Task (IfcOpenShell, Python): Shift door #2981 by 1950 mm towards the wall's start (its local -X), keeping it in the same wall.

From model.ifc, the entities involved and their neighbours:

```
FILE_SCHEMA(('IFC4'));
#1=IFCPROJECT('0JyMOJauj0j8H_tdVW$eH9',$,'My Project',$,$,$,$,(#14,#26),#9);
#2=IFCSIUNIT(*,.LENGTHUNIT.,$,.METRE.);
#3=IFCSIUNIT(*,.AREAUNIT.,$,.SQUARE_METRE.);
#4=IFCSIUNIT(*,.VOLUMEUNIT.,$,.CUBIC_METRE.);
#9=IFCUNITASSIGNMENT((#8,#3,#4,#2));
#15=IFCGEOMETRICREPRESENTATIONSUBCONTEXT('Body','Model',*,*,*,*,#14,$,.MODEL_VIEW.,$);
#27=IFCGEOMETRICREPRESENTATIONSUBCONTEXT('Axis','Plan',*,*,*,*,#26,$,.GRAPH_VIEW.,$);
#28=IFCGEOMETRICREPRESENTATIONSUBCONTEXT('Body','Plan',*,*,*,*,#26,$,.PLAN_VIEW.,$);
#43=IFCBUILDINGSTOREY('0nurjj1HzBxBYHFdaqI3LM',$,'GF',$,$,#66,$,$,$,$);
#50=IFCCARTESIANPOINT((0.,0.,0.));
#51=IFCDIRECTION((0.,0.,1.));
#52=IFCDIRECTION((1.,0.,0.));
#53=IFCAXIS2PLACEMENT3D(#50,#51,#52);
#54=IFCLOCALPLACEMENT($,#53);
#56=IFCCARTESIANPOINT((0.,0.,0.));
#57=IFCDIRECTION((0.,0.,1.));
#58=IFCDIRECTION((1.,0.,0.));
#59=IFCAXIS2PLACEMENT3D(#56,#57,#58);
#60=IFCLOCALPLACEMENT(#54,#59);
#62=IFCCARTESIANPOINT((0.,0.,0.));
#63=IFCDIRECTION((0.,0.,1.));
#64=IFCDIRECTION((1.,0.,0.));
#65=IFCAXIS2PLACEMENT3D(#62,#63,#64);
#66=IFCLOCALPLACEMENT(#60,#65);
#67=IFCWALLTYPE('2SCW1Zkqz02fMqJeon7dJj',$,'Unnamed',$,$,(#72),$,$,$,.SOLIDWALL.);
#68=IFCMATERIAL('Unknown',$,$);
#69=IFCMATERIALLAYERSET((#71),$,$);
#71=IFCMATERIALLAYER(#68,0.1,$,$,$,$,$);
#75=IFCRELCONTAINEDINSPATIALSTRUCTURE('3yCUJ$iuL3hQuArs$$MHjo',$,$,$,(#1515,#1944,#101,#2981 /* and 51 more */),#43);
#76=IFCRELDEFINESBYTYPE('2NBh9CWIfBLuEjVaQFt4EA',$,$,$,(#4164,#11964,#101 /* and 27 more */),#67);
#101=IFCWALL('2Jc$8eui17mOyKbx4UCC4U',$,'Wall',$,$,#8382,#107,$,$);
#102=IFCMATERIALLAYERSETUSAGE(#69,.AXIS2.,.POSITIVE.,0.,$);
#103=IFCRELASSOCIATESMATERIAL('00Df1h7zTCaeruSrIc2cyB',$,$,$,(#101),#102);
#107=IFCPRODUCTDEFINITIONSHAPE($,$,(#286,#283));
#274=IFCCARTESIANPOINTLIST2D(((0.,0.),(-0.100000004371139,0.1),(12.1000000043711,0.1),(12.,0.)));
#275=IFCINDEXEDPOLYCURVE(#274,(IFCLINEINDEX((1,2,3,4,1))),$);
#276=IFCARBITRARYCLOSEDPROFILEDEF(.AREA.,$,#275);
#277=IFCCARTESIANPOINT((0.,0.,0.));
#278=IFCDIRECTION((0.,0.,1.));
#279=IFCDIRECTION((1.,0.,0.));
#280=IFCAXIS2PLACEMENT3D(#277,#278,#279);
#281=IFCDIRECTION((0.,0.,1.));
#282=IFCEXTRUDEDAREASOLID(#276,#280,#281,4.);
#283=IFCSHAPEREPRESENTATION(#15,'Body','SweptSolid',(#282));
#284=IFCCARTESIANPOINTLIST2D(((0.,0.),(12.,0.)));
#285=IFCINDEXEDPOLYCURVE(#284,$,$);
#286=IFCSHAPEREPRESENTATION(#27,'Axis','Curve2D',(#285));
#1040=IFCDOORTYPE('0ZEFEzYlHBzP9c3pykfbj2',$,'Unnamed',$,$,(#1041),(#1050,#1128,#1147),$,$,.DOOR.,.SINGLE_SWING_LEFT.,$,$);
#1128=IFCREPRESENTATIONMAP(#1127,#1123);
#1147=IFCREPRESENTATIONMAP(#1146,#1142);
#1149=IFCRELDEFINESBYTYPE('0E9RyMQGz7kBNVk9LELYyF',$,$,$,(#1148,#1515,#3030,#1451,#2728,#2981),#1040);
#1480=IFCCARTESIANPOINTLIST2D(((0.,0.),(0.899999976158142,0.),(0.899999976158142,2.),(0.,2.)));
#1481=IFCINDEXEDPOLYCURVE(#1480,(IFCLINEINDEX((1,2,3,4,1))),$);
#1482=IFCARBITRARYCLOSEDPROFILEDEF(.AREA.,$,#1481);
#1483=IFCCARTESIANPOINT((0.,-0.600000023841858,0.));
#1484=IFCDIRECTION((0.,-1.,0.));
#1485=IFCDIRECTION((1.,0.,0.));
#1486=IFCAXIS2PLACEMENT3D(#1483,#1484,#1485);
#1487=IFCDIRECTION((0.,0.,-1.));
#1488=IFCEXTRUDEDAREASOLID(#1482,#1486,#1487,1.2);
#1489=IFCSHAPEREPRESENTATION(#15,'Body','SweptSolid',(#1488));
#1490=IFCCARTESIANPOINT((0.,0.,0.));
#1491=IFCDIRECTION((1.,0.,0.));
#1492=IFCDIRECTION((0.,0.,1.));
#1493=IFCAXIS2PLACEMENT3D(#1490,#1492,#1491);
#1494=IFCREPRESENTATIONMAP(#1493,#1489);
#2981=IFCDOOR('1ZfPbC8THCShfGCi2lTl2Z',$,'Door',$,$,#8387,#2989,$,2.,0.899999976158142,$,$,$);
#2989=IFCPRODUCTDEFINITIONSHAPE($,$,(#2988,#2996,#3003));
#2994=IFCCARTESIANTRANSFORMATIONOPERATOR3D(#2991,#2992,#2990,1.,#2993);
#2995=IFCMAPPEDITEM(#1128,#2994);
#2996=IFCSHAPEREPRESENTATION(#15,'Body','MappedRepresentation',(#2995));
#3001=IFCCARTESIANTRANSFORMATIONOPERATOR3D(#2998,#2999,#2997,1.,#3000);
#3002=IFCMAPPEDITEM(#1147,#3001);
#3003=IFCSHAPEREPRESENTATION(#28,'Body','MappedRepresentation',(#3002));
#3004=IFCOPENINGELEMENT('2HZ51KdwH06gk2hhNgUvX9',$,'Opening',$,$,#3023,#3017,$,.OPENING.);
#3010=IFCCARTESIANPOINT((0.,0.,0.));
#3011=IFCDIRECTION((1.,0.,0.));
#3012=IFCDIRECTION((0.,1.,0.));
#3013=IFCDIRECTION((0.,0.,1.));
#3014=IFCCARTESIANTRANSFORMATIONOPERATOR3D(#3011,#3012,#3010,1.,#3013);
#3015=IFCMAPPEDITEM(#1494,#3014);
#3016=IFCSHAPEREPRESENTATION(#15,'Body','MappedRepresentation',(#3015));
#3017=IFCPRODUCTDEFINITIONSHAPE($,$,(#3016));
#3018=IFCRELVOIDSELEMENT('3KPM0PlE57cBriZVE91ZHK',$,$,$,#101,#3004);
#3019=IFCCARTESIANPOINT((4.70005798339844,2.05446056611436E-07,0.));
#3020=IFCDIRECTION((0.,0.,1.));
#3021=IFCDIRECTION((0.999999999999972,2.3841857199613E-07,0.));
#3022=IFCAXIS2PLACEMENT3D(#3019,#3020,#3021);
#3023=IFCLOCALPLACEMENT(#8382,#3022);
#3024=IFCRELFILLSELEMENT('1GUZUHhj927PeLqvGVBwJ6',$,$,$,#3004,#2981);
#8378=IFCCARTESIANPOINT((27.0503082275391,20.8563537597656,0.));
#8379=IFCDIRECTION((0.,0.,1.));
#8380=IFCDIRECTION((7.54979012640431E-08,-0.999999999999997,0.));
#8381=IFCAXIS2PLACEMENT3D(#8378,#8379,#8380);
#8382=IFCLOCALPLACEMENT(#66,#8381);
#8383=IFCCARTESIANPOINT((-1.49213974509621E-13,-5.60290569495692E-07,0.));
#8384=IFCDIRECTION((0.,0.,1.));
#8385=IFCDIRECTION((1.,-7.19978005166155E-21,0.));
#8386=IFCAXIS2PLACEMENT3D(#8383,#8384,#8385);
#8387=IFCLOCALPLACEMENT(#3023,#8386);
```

```python
import ifcopenshell
import ifcopenshell.api.geometry
import ifcopenshell.util.placement
import ifcopenshell.util.unit

model = ifcopenshell.open("model.ifc")
unit_scale = ifcopenshell.util.unit.calculate_unit_scale(model)

door = model.by_guid("1ZfPbC8THCShfGCi2lTl2Z")
opening = door.FillsVoids[0].RelatingOpeningElement
wall = opening.VoidsElements[0].RelatingBuildingElement

wall_matrix = ifcopenshell.util.placement.get_local_placement(wall.ObjectPlacement)
shift = wall_matrix[:3, 0] * -1.95 / unit_scale
before = ifcopenshell.util.placement.get_local_placement(door.ObjectPlacement)[:3, 3].copy()

# The door is placed relative to its opening, so it follows when the opening moves.
matrix = ifcopenshell.util.placement.get_local_placement(opening.ObjectPlacement)
matrix[:3, 3] += shift
ifcopenshell.api.geometry.edit_object_placement(
    model, product=opening, matrix=matrix, is_si=False, should_transform_children=True
)

after = ifcopenshell.util.placement.get_local_placement(door.ObjectPlacement)[:3, 3]
print("door moved by", (after - before).round(3) + 0.0)

model.write("model_v2.ifc")
```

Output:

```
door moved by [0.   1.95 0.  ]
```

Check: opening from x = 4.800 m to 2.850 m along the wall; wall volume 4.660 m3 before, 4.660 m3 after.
